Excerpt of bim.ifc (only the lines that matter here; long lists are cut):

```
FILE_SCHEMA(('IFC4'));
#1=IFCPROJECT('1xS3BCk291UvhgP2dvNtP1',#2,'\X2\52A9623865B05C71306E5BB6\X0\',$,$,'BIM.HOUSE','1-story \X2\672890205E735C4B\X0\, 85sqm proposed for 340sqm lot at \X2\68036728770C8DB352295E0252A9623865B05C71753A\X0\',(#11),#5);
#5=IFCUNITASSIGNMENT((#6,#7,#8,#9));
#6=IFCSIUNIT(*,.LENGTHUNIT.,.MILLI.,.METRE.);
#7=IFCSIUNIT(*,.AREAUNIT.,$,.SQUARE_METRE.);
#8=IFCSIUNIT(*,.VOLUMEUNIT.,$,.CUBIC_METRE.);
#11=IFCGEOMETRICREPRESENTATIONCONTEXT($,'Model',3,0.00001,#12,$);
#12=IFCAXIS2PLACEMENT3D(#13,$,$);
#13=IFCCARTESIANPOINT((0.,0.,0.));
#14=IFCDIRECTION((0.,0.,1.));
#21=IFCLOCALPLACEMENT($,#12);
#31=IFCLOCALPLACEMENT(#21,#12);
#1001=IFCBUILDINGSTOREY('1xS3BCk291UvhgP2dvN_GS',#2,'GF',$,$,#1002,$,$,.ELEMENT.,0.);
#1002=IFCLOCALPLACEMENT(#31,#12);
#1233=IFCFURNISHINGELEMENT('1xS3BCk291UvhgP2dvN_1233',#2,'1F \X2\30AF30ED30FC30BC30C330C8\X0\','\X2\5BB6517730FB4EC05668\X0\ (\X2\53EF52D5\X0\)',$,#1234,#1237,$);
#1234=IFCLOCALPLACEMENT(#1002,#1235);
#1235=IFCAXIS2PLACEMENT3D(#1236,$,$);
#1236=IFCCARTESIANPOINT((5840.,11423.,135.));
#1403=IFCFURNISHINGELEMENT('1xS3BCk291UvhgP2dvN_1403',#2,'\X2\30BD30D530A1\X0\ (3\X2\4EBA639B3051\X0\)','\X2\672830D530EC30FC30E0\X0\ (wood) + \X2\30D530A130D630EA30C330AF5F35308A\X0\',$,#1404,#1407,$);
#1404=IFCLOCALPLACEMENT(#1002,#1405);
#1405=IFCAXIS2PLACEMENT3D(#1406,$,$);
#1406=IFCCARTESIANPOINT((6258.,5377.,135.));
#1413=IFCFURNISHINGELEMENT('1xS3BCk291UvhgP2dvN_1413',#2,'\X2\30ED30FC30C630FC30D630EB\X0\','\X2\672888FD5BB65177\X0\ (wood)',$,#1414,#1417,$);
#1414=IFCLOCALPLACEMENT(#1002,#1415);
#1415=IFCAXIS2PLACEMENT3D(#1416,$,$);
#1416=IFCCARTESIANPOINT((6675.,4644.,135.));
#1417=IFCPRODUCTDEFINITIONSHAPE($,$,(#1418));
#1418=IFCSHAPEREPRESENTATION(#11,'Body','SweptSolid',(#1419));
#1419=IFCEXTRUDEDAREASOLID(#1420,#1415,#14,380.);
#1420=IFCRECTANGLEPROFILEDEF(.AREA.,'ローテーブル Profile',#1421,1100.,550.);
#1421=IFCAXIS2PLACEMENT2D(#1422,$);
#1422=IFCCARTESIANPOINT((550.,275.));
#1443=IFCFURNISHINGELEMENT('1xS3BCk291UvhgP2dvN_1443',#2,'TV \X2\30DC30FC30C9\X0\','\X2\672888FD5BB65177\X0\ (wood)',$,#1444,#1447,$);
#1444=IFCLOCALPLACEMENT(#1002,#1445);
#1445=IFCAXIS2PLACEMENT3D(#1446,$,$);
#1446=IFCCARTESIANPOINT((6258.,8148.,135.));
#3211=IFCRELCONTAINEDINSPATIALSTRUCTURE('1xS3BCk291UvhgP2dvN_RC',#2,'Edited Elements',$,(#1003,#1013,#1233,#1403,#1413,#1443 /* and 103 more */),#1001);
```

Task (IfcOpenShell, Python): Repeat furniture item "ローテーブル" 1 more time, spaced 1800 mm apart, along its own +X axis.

```python
import ifcopenshell
import ifcopenshell.api.geometry
import ifcopenshell.api.root
import ifcopenshell.util.element
import ifcopenshell.util.placement
import ifcopenshell.util.unit

model = ifcopenshell.open("bim.ifc")
unit_scale = ifcopenshell.util.unit.calculate_unit_scale(model)


def reuse_history(source, copy):
    """copy_class also copies each property set's owner history, people and application; keep the originals."""
    for rel in copy.IsDefinedBy:
        if rel.is_a("IfcRelDefinesByProperties") and (history := rel.RelatingPropertyDefinition.OwnerHistory):
            rel.RelatingPropertyDefinition.OwnerHistory = source.OwnerHistory
            ifcopenshell.util.element.remove_deep2(model, history)


source = model.by_guid("1xS3BCk291UvhgP2dvN_1413")
base = ifcopenshell.util.placement.get_local_placement(source.ObjectPlacement)
step = base[:3, 0] * 1.8 / unit_scale

for i in range(1, 2):
    copy = ifcopenshell.api.root.copy_class(model, product=source)
    copy.Representation = ifcopenshell.util.element.copy_deep(
        model, source.Representation, exclude=["IfcGeometricRepresentationContext", "IfcRepresentationMap"]
    )
    reuse_history(source, copy)
    matrix = base.copy()
    matrix[:3, 3] += i * step
    print("added at", matrix[:3, 3].round(3) + 0.0)
    ifcopenshell.api.geometry.edit_object_placement(model, product=copy, matrix=matrix, is_si=False)

model.write("bim_updated.ifc")
```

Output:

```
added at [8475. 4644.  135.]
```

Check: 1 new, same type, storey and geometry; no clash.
